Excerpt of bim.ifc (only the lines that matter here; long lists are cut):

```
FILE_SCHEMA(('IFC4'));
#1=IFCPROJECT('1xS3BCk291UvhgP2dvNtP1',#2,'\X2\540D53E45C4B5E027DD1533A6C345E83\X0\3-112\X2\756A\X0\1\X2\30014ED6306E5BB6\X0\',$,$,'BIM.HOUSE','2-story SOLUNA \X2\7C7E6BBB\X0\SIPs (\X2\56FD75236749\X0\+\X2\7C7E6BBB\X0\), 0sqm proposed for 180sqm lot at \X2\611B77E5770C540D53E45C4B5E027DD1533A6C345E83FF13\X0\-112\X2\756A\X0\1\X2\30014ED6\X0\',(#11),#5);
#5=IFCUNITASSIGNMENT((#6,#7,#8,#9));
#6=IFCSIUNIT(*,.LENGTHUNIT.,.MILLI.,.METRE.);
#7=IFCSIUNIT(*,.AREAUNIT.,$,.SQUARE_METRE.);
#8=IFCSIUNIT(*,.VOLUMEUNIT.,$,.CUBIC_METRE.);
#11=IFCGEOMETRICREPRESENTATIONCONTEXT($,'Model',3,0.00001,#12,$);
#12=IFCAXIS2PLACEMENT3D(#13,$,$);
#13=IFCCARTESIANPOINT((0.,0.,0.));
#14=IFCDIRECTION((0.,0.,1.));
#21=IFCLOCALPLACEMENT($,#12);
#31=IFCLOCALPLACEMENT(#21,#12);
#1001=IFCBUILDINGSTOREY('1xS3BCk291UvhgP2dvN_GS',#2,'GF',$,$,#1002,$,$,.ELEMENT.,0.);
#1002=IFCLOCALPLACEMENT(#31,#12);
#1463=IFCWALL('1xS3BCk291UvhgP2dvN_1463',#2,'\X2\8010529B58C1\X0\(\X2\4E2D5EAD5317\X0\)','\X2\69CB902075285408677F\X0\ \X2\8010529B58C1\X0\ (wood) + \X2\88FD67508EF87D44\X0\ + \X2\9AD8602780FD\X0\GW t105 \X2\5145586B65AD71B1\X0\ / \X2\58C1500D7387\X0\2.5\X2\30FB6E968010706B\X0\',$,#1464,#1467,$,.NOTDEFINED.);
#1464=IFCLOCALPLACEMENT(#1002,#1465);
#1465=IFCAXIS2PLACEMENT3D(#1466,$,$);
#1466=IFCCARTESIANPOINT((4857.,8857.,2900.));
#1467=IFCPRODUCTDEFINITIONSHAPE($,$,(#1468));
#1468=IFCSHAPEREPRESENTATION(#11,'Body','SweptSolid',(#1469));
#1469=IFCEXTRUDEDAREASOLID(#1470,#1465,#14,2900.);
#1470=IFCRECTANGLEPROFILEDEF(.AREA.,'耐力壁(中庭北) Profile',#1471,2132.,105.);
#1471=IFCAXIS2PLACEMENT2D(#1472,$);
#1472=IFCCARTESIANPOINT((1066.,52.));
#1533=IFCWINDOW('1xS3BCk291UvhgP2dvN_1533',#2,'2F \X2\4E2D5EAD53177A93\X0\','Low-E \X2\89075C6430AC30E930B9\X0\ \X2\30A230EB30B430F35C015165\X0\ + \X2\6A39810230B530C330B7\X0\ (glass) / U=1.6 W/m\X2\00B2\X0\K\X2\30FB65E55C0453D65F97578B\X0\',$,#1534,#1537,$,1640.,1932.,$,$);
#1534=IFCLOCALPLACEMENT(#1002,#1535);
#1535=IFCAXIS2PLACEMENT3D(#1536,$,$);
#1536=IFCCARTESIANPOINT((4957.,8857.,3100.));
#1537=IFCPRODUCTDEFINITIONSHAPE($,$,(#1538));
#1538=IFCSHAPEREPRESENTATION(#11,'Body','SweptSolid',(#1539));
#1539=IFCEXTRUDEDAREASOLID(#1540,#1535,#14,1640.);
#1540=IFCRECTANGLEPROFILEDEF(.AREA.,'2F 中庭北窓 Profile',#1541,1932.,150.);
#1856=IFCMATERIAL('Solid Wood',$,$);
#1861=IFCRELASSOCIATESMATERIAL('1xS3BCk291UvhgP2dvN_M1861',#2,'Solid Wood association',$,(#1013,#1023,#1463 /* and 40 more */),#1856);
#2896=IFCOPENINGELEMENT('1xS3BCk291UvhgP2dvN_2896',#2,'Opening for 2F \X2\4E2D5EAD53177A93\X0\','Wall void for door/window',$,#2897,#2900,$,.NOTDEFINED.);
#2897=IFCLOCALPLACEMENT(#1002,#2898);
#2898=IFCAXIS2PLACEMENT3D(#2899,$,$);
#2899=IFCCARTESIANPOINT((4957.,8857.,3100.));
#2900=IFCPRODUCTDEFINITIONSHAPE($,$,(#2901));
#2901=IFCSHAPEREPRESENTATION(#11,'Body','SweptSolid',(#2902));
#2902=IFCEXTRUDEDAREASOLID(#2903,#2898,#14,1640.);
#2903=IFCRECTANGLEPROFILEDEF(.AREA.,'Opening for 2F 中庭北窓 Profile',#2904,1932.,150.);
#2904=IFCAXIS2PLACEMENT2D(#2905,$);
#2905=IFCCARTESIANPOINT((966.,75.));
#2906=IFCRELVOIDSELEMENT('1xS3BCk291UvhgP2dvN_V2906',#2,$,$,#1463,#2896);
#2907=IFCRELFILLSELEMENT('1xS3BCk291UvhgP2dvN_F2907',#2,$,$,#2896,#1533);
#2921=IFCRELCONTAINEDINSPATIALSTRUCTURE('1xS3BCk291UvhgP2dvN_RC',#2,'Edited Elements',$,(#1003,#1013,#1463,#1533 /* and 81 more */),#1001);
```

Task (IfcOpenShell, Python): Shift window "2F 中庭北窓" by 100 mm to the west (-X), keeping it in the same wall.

```python
import ifcopenshell
import ifcopenshell.api.geometry
import ifcopenshell.util.placement
import ifcopenshell.util.unit

model = ifcopenshell.open("bim.ifc")
unit_scale = ifcopenshell.util.unit.calculate_unit_scale(model)

window = model.by_id(1533)
opening = window.FillsVoids[0].RelatingOpeningElement
wall = opening.VoidsElements[0].RelatingBuildingElement

wall_matrix = ifcopenshell.util.placement.get_local_placement(wall.ObjectPlacement)
shift = wall_matrix[:3, 0] * -0.1 / unit_scale
before = ifcopenshell.util.placement.get_local_placement(window.ObjectPlacement)[:3, 3].copy()

# The window is not placed relative to its opening, so move both.
for product in (opening, window):
    matrix = ifcopenshell.util.placement.get_local_placement(product.ObjectPlacement)
    matrix[:3, 3] += shift
    ifcopenshell.api.geometry.edit_object_placement(model, product=product, matrix=matrix, is_si=False)

after = ifcopenshell.util.placement.get_local_placement(window.ObjectPlacement)[:3, 3]
print("window moved by", (after - before).round(3) + 0.0)

model.write("bim_updated.ifc")
```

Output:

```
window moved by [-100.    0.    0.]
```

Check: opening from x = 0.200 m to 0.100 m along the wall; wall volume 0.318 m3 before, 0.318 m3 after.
